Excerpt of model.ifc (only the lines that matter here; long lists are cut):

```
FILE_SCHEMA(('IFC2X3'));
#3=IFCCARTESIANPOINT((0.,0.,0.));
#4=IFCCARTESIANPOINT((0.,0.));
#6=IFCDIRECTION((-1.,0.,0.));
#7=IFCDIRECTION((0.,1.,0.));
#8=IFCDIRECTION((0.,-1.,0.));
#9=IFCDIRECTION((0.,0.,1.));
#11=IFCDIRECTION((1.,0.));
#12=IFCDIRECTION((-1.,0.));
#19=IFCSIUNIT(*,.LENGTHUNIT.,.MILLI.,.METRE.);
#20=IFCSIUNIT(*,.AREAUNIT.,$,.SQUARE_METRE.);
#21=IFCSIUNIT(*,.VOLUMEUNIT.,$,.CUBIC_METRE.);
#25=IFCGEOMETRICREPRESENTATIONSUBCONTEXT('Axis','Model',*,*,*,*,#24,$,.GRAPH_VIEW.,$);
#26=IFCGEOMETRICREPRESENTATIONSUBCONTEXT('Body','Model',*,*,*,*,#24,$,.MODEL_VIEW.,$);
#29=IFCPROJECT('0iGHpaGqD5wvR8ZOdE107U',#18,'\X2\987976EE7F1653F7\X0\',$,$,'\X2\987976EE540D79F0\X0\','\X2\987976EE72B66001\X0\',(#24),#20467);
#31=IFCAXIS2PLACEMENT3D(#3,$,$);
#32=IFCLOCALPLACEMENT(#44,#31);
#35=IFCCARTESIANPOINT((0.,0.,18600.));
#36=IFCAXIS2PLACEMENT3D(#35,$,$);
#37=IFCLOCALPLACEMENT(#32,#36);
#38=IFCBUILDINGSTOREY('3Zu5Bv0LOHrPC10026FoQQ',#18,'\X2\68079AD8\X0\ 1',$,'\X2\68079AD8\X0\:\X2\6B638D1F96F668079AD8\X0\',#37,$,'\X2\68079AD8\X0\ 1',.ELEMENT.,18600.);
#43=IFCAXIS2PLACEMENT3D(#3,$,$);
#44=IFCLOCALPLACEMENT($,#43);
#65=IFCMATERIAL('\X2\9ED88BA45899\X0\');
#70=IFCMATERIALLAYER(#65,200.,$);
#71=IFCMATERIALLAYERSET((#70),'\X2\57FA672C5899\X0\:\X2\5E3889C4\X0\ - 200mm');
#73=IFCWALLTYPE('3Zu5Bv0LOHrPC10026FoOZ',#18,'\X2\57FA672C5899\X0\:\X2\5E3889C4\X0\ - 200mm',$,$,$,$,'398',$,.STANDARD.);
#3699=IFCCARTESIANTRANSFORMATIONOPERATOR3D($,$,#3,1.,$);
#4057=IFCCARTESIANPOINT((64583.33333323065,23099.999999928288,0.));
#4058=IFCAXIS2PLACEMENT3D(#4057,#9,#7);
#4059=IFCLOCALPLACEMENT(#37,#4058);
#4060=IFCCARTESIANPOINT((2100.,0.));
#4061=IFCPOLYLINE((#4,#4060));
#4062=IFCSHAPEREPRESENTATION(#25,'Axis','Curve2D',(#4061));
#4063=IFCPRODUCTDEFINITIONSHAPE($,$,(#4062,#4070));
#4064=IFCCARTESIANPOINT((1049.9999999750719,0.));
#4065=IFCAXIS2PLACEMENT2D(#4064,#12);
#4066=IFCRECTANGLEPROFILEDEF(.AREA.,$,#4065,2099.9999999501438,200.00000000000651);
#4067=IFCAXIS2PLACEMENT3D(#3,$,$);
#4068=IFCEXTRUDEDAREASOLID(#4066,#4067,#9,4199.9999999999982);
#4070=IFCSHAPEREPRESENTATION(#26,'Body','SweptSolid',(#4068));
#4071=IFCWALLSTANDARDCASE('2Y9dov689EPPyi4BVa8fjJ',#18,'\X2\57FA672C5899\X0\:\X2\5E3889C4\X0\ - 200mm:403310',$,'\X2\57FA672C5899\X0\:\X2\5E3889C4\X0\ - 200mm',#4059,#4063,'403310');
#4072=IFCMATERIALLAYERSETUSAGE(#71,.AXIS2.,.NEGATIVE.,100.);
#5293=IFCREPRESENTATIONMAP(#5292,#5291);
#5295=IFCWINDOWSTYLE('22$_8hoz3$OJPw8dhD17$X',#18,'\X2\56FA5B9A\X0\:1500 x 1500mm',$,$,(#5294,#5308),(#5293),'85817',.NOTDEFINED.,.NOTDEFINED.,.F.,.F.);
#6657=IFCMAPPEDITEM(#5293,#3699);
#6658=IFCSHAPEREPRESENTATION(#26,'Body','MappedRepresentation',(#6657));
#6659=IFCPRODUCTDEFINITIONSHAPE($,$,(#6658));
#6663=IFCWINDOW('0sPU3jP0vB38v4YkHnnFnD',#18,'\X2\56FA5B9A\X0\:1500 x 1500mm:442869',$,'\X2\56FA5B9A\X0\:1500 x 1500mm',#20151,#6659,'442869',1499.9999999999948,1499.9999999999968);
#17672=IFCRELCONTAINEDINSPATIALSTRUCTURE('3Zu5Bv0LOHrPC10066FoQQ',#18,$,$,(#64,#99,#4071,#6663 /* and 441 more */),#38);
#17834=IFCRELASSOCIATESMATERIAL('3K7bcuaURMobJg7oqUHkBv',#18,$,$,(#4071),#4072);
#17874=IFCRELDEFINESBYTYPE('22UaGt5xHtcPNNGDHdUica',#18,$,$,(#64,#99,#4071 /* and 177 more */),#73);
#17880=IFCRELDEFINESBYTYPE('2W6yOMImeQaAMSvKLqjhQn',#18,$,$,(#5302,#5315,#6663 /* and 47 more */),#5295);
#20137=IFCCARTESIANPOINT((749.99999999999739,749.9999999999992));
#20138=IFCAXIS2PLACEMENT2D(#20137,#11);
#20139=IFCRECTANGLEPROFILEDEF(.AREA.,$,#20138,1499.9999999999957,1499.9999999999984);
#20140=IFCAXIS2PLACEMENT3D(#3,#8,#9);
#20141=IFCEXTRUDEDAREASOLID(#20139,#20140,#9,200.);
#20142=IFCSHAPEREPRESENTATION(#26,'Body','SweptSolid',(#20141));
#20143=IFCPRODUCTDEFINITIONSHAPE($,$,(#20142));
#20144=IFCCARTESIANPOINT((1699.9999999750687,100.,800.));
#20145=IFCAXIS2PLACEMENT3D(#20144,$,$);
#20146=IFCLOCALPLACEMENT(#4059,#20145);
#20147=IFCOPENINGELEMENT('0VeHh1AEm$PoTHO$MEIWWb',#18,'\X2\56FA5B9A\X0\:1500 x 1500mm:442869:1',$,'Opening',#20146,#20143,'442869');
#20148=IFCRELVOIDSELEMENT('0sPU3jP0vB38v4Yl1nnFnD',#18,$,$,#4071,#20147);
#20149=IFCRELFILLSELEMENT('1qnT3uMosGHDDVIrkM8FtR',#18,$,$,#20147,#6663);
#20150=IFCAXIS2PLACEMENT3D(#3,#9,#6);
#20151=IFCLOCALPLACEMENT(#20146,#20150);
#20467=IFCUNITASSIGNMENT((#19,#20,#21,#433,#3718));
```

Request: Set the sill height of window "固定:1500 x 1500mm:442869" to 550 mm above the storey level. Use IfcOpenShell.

```python
import numpy as np
import ifcopenshell
import ifcopenshell.api.geometry
import ifcopenshell.geom
import ifcopenshell.util.element
import ifcopenshell.util.placement
import ifcopenshell.util.shape
import ifcopenshell.util.unit

model = ifcopenshell.open("model.ifc")
unit_scale = ifcopenshell.util.unit.calculate_unit_scale(model)

window = model.by_guid("0sPU3jP0vB38v4YkHnnFnD")
opening = window.FillsVoids[0].RelatingOpeningElement
storey = ifcopenshell.util.element.get_container(window, ifc_class="IfcBuildingStorey")
level = ifcopenshell.util.placement.get_local_placement(storey.ObjectPlacement)[2, 3]

# The opening's origin need not be at the sill, so measure its lowest point.
shape = ifcopenshell.geom.create_shape(ifcopenshell.geom.settings(), opening)
bottom = ifcopenshell.util.shape.get_shape_bottom_elevation(shape, shape.geometry) / unit_scale
dz = level + 550.0 - bottom

shift = np.array([0.0, 0.0, dz])
# The window is placed relative to its opening, so it follows when the opening moves.
matrix = ifcopenshell.util.placement.get_local_placement(opening.ObjectPlacement)
matrix[:3, 3] += shift
ifcopenshell.api.geometry.edit_object_placement(
    model, product=opening, matrix=matrix, is_si=False, should_transform_children=True
)

print(f"moved by {dz * unit_scale:+.3f} m")

model.write("model-out.ifc")
```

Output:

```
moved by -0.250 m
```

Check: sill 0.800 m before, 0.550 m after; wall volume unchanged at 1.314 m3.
